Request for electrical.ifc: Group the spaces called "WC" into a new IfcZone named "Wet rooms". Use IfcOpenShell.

First a look at what the model holds.

```python
import ifcopenshell

model = ifcopenshell.open("electrical.ifc")
print(model.schema)
seen = {}
for space in model.by_type("IfcSpace"):
    seen[space.LongName] = seen.get(space.LongName, 0) + 1
for name, count in sorted(seen.items(), key=str):
    print(count, "x", name)
print("zones:", [z.Name for z in model.by_type("IfcZone")][:20])
```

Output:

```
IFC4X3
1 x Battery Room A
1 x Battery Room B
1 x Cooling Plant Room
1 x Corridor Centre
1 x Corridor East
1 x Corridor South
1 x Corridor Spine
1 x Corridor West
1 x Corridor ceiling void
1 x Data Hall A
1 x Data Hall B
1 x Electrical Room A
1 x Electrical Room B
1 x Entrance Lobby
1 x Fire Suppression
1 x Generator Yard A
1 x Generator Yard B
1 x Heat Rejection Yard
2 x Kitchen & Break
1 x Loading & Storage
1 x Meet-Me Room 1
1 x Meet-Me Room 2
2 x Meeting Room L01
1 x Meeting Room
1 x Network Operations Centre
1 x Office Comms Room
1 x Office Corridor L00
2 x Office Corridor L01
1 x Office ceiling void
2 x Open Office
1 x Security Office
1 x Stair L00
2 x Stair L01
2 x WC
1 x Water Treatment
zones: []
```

```python
import ifcopenshell
import ifcopenshell.api.group
import ifcopenshell.api.root

model = ifcopenshell.open("electrical.ifc")

names = {"WC"}
spaces = [s for s in model.by_type("IfcSpace") if s.LongName in names]

zone = ifcopenshell.api.root.create_entity(model, ifc_class="IfcZone", name="Wet rooms")
ifcopenshell.api.group.assign_group(model, products=spaces, group=zone)
print(len(spaces), "spaces in", zone.Name)

model.write("electrical_rev.ifc")
```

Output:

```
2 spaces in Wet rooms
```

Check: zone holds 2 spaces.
